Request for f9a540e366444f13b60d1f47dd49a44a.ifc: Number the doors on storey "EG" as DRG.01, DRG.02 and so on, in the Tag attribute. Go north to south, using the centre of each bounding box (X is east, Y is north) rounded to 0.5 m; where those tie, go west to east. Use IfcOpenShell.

First a look at what the model holds.

```python
import ifcopenshell
import ifcopenshell.util.element
import ifcopenshell.util.placement

model = ifcopenshell.open("f9a540e366444f13b60d1f47dd49a44a.ifc")
print(model.schema)
storey = next(s for s in model.by_type("IfcBuildingStorey") if s.Name == "EG")
doors = [e for e in ifcopenshell.util.element.get_decomposition(storey) if e.is_a("IfcDoor")]
for e in sorted(doors, key=lambda e: e.id()):
    origin = ifcopenshell.util.placement.get_local_placement(e.ObjectPlacement)[:3, 3]
    print(e.id(), e.Tag, e.Name, origin.round(2) + 0.0, sep=" | ")
```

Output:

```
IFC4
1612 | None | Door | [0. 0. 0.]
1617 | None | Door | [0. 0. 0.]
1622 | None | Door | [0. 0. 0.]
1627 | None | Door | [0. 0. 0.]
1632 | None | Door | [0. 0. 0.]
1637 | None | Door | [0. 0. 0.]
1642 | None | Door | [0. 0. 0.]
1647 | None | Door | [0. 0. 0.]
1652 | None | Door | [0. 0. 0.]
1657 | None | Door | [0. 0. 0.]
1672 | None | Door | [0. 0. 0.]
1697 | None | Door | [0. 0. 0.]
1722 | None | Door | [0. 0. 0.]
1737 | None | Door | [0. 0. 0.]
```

```python
import ifcopenshell
import ifcopenshell.geom
import ifcopenshell.util.element
import ifcopenshell.util.shape

model = ifcopenshell.open("f9a540e366444f13b60d1f47dd49a44a.ifc")
settings = ifcopenshell.geom.settings()
settings.set("use-world-coords", True)


def centre(element):
    shape = ifcopenshell.geom.create_shape(settings, element)
    return ifcopenshell.util.shape.get_bbox_centroid(shape.geometry)


storey = next(s for s in model.by_type("IfcBuildingStorey") if s.Name == "EG")
doors = [e for e in ifcopenshell.util.element.get_decomposition(storey) if e.is_a("IfcDoor")]

# Insertion points can sit at a corner or the storey origin, so sort by the geometry (in metres).
centres = {e: centre(e) for e in doors}
doors.sort(key=lambda e: (-round(centres[e][1] / 0.5), centres[e][0]))

for i, e in enumerate(doors, start=1):
    number = f"DRG.{i:02d}"
    e.Tag = number
    print(e.id(), number)

model.write("f9a540e366444f13b60d1f47dd49a44a-out.ifc")
```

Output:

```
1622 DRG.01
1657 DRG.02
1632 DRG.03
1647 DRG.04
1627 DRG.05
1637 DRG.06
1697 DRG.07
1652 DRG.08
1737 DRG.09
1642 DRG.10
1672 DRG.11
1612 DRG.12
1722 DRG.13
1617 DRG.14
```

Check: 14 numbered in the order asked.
